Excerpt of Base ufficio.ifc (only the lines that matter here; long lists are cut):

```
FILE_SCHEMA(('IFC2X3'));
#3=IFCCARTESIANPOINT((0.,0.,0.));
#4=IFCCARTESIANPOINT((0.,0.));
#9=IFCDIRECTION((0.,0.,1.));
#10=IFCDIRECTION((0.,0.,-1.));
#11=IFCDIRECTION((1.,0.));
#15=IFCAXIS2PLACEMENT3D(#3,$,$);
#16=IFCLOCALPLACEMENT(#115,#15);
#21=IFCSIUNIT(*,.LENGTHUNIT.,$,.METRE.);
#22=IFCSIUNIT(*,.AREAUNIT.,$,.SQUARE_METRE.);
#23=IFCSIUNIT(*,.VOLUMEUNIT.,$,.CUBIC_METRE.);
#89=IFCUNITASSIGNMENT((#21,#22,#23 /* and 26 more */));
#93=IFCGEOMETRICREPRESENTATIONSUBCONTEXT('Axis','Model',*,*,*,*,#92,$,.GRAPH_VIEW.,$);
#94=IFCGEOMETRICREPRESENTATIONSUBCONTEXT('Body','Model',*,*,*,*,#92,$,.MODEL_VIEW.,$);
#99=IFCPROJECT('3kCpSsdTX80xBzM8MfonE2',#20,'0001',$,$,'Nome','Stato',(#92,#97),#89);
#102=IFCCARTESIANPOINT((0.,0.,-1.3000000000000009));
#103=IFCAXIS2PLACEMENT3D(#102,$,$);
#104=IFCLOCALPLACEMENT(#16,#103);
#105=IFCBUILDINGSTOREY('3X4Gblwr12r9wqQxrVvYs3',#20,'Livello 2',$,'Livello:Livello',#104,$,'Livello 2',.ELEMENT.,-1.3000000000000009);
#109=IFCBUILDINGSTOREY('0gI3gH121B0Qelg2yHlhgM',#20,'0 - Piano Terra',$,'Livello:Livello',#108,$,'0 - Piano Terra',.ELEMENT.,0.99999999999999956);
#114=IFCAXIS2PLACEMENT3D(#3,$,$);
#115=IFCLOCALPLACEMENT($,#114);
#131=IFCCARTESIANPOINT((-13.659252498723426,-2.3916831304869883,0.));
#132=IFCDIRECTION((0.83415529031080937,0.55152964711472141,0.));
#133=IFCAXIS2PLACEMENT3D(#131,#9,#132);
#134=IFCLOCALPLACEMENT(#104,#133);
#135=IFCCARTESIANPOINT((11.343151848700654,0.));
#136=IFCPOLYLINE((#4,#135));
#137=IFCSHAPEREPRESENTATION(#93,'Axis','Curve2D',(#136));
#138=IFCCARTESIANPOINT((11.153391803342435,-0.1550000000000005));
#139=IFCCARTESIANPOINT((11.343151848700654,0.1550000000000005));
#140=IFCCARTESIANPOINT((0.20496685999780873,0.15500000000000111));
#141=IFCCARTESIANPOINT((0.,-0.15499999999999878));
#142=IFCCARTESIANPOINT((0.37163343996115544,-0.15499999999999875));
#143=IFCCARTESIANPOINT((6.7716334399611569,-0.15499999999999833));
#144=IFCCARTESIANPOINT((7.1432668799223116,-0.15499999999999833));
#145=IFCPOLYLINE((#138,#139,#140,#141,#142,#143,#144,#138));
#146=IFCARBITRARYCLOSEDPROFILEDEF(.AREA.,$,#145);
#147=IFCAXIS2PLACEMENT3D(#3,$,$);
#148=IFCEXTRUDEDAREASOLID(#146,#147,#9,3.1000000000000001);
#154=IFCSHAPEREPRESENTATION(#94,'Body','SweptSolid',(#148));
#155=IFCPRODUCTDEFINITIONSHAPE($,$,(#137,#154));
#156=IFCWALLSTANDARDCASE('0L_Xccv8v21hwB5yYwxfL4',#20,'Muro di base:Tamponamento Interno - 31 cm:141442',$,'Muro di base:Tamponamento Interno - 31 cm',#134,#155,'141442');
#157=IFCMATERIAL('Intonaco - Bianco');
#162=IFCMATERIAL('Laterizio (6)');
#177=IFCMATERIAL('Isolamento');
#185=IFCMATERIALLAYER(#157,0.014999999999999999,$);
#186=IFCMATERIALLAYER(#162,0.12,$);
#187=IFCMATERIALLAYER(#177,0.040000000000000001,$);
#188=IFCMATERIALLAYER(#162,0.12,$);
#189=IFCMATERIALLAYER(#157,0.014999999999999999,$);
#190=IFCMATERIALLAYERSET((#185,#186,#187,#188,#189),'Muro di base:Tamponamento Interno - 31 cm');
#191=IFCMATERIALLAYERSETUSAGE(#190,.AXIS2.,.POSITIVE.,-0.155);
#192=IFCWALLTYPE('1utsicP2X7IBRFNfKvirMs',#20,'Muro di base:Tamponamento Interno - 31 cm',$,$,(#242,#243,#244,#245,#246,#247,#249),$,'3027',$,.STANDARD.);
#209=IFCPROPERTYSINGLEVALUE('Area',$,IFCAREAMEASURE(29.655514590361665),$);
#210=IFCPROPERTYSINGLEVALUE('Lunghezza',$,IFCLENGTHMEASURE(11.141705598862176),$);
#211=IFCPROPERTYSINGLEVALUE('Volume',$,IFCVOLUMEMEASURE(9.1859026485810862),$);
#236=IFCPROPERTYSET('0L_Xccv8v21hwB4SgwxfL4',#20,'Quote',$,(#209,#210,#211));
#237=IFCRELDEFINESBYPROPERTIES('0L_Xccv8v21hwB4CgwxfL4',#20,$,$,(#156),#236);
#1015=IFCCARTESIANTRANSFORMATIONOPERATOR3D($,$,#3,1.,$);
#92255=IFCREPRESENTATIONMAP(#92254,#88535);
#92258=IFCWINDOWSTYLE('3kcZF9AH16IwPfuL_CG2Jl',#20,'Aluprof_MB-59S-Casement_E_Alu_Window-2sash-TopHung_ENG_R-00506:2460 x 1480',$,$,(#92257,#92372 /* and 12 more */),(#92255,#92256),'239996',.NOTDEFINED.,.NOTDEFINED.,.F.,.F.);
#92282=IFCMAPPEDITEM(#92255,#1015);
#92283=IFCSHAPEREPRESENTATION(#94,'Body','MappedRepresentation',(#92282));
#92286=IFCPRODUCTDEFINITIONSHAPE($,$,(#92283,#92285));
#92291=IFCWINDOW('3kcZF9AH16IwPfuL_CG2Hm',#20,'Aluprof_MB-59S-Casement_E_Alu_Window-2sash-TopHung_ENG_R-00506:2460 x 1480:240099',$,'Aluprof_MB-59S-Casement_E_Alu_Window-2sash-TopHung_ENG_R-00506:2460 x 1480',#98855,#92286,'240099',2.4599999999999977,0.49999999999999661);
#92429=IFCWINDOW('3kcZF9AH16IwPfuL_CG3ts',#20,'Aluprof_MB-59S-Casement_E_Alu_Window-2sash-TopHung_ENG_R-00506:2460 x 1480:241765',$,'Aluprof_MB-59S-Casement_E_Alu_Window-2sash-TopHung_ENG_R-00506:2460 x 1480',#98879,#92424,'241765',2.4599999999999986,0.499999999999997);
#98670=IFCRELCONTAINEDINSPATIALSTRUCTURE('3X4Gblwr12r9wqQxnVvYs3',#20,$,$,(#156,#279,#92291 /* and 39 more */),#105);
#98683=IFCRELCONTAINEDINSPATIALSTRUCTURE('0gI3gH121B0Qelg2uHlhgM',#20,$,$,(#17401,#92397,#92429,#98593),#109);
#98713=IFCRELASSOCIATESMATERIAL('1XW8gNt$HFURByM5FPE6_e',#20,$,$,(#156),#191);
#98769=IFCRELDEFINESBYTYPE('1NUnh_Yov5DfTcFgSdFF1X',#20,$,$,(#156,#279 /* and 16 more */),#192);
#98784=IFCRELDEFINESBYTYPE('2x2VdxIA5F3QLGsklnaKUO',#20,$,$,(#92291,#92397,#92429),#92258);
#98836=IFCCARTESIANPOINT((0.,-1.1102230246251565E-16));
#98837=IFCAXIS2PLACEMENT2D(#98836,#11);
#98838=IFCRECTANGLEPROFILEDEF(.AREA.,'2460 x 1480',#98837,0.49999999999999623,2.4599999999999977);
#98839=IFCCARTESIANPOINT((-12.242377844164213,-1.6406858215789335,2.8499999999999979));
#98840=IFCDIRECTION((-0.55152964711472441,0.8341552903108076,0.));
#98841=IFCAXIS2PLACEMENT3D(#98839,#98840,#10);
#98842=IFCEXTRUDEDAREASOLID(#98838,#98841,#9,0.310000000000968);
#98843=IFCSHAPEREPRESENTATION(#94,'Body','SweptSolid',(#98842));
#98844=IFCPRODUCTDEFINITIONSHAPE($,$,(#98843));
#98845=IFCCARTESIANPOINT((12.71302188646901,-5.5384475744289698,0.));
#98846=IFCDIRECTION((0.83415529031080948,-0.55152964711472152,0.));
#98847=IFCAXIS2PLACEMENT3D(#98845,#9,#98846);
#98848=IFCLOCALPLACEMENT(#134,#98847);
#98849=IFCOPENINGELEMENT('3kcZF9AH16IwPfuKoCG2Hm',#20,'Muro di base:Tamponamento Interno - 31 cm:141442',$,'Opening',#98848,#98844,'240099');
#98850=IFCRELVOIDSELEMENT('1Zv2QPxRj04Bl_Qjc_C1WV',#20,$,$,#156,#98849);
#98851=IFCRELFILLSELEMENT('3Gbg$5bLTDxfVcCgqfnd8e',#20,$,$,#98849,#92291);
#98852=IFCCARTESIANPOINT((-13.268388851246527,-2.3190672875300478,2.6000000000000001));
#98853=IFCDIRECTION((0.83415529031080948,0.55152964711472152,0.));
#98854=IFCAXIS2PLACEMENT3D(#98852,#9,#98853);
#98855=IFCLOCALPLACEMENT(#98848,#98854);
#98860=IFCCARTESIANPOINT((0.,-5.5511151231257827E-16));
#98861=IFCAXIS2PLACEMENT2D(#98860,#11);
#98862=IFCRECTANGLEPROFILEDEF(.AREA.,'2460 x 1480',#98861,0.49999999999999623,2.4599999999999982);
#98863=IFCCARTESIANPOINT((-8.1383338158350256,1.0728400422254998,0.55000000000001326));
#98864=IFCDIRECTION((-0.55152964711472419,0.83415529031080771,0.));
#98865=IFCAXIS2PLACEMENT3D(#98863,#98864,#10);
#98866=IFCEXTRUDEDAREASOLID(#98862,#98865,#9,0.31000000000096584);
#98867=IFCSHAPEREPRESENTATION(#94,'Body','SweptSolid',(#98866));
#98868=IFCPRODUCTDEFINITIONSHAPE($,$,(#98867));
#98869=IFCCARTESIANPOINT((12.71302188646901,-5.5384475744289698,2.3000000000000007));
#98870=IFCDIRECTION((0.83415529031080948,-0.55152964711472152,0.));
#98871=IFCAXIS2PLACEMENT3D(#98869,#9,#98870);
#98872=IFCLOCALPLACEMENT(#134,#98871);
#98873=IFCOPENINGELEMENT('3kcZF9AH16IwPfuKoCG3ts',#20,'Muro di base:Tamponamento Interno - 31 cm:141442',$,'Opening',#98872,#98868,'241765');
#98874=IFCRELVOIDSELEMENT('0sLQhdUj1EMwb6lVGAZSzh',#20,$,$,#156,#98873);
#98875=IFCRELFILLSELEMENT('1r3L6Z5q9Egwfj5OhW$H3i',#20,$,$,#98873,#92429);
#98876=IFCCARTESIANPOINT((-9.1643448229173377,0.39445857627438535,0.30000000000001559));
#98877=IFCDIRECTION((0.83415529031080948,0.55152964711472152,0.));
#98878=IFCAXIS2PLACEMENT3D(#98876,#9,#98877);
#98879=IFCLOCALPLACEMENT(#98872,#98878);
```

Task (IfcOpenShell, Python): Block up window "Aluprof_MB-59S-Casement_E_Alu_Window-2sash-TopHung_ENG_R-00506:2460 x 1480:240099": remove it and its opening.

```python
import ifcopenshell
import ifcopenshell.api.feature
import ifcopenshell.api.pset
import ifcopenshell.api.root
import ifcopenshell.geom
import ifcopenshell.util.element
import ifcopenshell.util.shape
import ifcopenshell.util.unit

model = ifcopenshell.open("Base ufficio.ifc")
area_scale = ifcopenshell.util.unit.calculate_unit_scale(model, "AREAUNIT")
volume_scale = ifcopenshell.util.unit.calculate_unit_scale(model, "VOLUMEUNIT")
settings = ifcopenshell.geom.settings()


def volume(element):
    """Net volume in cubic metres, openings subtracted."""
    shape = ifcopenshell.geom.create_shape(settings, element)
    return ifcopenshell.util.shape.get_volume(shape.geometry)


window = model.by_guid("3kcZF9AH16IwPfuL_CG2Hm")
opening = window.FillsVoids[0].RelatingOpeningElement
wall = opening.VoidsElements[0].RelatingBuildingElement
before = volume(wall)

ifcopenshell.api.root.remove_product(model, product=window)
ifcopenshell.api.feature.remove_feature(model, feature=opening)

after = volume(wall)
thickness = 0.31  # wall thickness in metres

# Update the wall's stored quantities.
pset = model.by_id(ifcopenshell.util.element.get_pset(wall, "Quote", should_inherit=False)["id"])
ifcopenshell.api.pset.edit_pset(model, pset=pset, properties={
    "Area": model.create_entity("IfcAreaMeasure", after / thickness / area_scale),
    "Volume": model.create_entity("IfcVolumeMeasure", after / volume_scale),
})

print(f"wall volume {before:.3f} -> {after:.3f} m3")

model.write("Base ufficio_v2.ifc")
```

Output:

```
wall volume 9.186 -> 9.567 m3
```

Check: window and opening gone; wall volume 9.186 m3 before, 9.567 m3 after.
